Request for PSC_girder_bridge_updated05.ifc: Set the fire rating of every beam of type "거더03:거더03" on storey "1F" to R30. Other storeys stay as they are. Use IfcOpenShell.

First a look at what the model holds.

```python
import ifcopenshell
import ifcopenshell.util.element

model = ifcopenshell.open("PSC_girder_bridge_updated05.ifc")
print(model.schema)
storey = next(s for s in model.by_type("IfcBuildingStorey") if s.Name == "1F")
beams = [e for e in ifcopenshell.util.element.get_decomposition(storey) if e.is_a("IfcBeam")]
seen = {}
for e in beams:
    element_type = ifcopenshell.util.element.get_type(e)
    key = (element_type.Name if element_type != e and element_type else None, ifcopenshell.util.element.get_pset(e, "Pset_BeamCommon", "FireRating"))
    seen[key] = seen.get(key, 0) + 1
for (name, value), count in sorted(seen.items(), key=str):
    print(count, "x", name, "|", value)
```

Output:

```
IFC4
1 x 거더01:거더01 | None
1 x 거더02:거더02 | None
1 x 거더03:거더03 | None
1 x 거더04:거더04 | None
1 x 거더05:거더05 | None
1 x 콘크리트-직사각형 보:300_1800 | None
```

```python
import ifcopenshell
import ifcopenshell.api.pset
import ifcopenshell.util.element

model = ifcopenshell.open("PSC_girder_bridge_updated05.ifc")

storey = next(s for s in model.by_type("IfcBuildingStorey") if s.Name == "1F")
beams = [e for e in ifcopenshell.util.element.get_decomposition(storey) if e.is_a("IfcBeam")]

count = 0
for e in beams:
    element_type = ifcopenshell.util.element.get_type(e)
    if element_type in (None, e) or element_type.Name != "거더03:거더03":
        continue
    # add_pset returns the element's existing set when there is one.
    pset = ifcopenshell.api.pset.add_pset(model, product=e, name="Pset_BeamCommon")
    ifcopenshell.api.pset.edit_pset(model, pset=pset, properties={"FireRating": "R30"})
    count += 1

print(count, "beams updated")

model.write("PSC_girder_bridge_updated05_rev.ifc")
```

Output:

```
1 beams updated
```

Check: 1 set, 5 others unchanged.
